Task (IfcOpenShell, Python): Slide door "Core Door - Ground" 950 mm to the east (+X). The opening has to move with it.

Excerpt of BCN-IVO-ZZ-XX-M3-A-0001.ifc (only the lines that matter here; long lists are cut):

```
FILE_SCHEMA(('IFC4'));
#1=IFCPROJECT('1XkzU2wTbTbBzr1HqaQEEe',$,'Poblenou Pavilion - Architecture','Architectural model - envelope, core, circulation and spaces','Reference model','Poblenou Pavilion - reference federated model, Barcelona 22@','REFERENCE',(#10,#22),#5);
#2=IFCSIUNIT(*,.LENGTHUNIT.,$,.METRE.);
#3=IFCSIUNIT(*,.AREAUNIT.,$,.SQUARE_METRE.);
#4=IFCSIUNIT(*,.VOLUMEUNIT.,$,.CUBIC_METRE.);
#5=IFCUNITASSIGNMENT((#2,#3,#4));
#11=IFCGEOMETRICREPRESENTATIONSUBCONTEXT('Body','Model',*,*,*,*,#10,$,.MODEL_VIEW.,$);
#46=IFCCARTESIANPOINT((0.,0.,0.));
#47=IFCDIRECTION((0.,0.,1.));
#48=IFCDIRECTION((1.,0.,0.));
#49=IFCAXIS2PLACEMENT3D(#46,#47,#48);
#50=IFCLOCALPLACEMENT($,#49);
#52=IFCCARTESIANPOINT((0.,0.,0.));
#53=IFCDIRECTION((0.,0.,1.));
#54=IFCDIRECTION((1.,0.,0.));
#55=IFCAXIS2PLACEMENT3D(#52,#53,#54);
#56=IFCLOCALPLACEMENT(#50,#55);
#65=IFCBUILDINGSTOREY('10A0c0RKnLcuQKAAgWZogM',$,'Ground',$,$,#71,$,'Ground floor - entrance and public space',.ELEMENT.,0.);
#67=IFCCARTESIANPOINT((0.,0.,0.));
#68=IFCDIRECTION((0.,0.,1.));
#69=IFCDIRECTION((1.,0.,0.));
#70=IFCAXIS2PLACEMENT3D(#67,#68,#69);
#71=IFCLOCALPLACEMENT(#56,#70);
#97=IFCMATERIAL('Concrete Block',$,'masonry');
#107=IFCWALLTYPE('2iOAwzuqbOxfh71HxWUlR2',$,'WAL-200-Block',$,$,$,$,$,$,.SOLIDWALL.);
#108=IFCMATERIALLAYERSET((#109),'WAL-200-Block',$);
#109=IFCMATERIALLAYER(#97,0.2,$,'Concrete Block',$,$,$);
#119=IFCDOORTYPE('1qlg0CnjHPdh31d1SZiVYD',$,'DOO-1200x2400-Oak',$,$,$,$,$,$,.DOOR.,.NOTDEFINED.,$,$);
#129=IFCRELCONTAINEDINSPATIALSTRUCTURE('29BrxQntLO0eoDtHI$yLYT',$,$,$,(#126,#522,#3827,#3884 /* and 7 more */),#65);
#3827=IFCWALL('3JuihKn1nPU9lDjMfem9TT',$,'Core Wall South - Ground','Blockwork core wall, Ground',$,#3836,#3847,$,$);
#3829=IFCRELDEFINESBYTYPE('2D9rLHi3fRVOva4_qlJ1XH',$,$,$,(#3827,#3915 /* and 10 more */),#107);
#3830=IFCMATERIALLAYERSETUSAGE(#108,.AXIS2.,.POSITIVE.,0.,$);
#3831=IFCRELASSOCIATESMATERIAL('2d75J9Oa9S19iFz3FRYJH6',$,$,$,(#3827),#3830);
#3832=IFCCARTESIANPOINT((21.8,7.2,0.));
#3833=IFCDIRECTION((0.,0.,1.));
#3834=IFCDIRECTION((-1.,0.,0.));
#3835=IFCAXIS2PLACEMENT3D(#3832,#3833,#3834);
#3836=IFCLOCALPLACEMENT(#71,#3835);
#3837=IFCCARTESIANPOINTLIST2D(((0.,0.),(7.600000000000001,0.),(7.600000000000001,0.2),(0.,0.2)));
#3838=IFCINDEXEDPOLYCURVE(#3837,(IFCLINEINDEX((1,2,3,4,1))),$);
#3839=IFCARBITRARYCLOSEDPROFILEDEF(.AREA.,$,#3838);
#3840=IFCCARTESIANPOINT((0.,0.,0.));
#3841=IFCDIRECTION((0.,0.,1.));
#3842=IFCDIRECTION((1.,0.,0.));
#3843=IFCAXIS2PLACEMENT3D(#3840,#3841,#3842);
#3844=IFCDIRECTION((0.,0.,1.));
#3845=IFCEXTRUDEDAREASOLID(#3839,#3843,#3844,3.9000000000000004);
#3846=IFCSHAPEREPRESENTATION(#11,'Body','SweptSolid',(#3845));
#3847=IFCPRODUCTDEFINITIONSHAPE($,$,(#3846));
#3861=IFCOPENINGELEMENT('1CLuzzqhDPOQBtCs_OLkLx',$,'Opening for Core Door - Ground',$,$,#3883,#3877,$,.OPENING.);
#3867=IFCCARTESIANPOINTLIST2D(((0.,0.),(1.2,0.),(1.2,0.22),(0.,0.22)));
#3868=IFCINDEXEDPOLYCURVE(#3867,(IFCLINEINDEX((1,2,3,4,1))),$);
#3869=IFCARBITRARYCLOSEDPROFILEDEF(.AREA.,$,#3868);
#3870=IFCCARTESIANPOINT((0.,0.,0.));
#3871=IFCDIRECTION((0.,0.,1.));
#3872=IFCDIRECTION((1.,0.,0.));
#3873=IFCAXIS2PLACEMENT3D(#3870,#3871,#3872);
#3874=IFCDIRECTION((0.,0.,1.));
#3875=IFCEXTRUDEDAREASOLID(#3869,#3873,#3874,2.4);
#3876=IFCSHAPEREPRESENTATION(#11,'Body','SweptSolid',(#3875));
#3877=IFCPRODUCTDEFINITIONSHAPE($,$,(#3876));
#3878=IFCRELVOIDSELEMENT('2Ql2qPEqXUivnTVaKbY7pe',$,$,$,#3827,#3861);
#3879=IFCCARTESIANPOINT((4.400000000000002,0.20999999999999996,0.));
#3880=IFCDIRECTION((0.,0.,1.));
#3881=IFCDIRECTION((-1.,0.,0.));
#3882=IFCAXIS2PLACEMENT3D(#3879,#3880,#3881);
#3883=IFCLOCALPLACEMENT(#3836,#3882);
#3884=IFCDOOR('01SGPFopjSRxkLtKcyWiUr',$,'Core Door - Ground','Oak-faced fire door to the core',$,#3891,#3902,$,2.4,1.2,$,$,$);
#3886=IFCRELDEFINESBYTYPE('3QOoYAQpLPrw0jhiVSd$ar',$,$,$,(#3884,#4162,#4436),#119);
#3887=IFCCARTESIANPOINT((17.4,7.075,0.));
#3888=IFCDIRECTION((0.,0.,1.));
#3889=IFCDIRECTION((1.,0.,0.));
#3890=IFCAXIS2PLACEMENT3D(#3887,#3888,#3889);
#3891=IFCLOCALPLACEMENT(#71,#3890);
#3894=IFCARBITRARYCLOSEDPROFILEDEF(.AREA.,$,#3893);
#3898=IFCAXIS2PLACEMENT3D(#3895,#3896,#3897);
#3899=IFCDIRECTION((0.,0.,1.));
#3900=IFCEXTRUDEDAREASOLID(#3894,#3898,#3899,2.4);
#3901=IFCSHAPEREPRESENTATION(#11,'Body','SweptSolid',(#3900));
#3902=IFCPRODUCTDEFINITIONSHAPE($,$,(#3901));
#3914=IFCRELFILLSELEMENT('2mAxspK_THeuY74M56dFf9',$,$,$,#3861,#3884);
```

```python
import ifcopenshell
import ifcopenshell.api.geometry
import ifcopenshell.util.placement
import ifcopenshell.util.unit

model = ifcopenshell.open("BCN-IVO-ZZ-XX-M3-A-0001.ifc")
unit_scale = ifcopenshell.util.unit.calculate_unit_scale(model)

door = model.by_guid("01SGPFopjSRxkLtKcyWiUr")
opening = door.FillsVoids[0].RelatingOpeningElement
wall = opening.VoidsElements[0].RelatingBuildingElement

wall_matrix = ifcopenshell.util.placement.get_local_placement(wall.ObjectPlacement)
shift = wall_matrix[:3, 0] * -0.95 / unit_scale
before = ifcopenshell.util.placement.get_local_placement(door.ObjectPlacement)[:3, 3].copy()

# The door is not placed relative to its opening, so move both.
for product in (opening, door):
    matrix = ifcopenshell.util.placement.get_local_placement(product.ObjectPlacement)
    matrix[:3, 3] += shift
    ifcopenshell.api.geometry.edit_object_placement(model, product=product, matrix=matrix, is_si=False)

after = ifcopenshell.util.placement.get_local_placement(door.ObjectPlacement)[:3, 3]
print("door moved by", (after - before).round(3) + 0.0)

model.write("BCN-IVO-ZZ-XX-M3-A-0001_updated.ifc")
```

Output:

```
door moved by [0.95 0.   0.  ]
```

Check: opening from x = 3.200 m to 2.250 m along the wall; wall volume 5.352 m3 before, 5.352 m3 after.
